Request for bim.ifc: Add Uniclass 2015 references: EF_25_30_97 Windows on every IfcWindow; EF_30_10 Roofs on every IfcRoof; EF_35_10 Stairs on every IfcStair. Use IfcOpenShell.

First a look at what the model holds.

```python
import ifcopenshell

model = ifcopenshell.open("bim.ifc")
print(model.schema)
print("classifications:", [c.Name for c in model.by_type("IfcClassification")])
for ifc_class in ("IfcDoor", "IfcRoof", "IfcStair", "IfcWall", "IfcWindow"):
    print(ifc_class, len(model.by_type(ifc_class)))
```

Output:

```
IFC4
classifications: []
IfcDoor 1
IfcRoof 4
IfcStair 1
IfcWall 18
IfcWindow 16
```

```python
import ifcopenshell
import ifcopenshell.api.classification

model = ifcopenshell.open("bim.ifc")

system = ifcopenshell.api.classification.add_classification(model, classification="Uniclass 2015")

codes = {
    "IfcWindow": ("EF_25_30_97", "Windows"),
    "IfcRoof": ("EF_30_10", "Roofs"),
    "IfcStair": ("EF_35_10", "Stairs"),
}
for ifc_class, (code, name) in codes.items():
    products = model.by_type(ifc_class)
    ifcopenshell.api.classification.add_reference(
        model, products=products, classification=system, identification=code, name=name
    )
    print(code, len(products))

model.write("bim_v2.ifc")
```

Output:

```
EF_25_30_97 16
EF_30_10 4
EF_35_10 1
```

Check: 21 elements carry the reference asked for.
